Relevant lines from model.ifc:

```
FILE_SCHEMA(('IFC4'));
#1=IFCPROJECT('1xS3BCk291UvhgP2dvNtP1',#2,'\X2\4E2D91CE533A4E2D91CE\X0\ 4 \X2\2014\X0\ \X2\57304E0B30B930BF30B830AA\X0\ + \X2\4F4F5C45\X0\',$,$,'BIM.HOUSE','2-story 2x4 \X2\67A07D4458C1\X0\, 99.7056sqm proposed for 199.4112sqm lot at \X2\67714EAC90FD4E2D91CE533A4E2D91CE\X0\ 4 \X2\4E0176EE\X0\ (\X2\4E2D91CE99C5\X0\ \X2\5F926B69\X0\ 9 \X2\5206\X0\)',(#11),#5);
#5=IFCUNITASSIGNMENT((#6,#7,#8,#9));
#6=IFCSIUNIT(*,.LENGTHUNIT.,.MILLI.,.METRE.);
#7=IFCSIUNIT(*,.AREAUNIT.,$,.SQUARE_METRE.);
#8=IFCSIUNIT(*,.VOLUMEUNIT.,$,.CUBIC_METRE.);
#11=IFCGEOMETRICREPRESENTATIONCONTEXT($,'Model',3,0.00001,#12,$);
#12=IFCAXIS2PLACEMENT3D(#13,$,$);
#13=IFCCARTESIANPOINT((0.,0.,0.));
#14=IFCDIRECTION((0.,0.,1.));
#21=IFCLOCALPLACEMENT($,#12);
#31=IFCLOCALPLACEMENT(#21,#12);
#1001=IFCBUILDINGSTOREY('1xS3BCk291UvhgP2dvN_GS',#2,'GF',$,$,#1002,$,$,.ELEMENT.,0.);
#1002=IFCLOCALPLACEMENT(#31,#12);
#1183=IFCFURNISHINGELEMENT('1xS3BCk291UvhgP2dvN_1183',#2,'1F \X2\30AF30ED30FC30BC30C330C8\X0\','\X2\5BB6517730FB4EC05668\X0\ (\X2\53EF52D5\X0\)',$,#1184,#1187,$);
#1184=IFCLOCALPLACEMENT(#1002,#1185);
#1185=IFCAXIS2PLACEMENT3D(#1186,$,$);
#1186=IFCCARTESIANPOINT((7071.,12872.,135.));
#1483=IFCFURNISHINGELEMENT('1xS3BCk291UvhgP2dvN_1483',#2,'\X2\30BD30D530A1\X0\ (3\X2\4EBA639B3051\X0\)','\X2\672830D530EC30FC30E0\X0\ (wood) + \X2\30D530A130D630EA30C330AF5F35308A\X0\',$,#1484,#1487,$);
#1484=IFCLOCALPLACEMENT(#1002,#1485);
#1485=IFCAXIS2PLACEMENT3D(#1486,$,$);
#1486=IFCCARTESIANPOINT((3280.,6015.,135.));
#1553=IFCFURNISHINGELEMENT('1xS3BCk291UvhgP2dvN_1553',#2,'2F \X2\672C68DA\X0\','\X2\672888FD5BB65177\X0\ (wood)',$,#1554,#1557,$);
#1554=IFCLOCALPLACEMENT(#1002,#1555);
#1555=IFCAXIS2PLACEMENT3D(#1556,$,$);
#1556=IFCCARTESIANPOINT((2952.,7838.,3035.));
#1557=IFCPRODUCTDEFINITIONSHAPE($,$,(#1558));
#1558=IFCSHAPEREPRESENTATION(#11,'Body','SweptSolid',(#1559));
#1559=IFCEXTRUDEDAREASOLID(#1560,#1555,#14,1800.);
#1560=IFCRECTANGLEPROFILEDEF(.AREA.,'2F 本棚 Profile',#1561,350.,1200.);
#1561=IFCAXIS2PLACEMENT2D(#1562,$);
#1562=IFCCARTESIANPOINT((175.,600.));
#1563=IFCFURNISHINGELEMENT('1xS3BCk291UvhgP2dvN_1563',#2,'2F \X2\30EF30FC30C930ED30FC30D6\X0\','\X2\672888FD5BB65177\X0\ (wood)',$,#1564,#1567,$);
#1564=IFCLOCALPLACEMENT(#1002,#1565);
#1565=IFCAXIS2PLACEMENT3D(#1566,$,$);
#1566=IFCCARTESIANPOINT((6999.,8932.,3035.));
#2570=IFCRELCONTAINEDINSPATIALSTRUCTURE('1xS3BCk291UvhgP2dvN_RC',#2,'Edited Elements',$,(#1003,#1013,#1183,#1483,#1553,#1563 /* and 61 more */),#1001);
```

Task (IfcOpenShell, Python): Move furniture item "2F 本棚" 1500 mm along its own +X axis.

```python
import ifcopenshell
import ifcopenshell.api.geometry
import ifcopenshell.util.placement

model = ifcopenshell.open("model.ifc")

item = model.by_guid("1xS3BCk291UvhgP2dvN_1553")
matrix = ifcopenshell.util.placement.get_local_placement(item.ObjectPlacement)
matrix[:3, 3] += matrix[:3, 0] * 1500.0
ifcopenshell.api.geometry.edit_object_placement(model, product=item, matrix=matrix, is_si=False)

print(ifcopenshell.util.placement.get_local_placement(item.ObjectPlacement).round(3) + 0.0)

model.write("model-out.ifc")
```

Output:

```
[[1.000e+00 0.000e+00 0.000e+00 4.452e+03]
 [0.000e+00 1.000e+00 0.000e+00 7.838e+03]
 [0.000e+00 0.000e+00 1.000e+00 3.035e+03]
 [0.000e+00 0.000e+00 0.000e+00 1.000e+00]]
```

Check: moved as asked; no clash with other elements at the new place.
